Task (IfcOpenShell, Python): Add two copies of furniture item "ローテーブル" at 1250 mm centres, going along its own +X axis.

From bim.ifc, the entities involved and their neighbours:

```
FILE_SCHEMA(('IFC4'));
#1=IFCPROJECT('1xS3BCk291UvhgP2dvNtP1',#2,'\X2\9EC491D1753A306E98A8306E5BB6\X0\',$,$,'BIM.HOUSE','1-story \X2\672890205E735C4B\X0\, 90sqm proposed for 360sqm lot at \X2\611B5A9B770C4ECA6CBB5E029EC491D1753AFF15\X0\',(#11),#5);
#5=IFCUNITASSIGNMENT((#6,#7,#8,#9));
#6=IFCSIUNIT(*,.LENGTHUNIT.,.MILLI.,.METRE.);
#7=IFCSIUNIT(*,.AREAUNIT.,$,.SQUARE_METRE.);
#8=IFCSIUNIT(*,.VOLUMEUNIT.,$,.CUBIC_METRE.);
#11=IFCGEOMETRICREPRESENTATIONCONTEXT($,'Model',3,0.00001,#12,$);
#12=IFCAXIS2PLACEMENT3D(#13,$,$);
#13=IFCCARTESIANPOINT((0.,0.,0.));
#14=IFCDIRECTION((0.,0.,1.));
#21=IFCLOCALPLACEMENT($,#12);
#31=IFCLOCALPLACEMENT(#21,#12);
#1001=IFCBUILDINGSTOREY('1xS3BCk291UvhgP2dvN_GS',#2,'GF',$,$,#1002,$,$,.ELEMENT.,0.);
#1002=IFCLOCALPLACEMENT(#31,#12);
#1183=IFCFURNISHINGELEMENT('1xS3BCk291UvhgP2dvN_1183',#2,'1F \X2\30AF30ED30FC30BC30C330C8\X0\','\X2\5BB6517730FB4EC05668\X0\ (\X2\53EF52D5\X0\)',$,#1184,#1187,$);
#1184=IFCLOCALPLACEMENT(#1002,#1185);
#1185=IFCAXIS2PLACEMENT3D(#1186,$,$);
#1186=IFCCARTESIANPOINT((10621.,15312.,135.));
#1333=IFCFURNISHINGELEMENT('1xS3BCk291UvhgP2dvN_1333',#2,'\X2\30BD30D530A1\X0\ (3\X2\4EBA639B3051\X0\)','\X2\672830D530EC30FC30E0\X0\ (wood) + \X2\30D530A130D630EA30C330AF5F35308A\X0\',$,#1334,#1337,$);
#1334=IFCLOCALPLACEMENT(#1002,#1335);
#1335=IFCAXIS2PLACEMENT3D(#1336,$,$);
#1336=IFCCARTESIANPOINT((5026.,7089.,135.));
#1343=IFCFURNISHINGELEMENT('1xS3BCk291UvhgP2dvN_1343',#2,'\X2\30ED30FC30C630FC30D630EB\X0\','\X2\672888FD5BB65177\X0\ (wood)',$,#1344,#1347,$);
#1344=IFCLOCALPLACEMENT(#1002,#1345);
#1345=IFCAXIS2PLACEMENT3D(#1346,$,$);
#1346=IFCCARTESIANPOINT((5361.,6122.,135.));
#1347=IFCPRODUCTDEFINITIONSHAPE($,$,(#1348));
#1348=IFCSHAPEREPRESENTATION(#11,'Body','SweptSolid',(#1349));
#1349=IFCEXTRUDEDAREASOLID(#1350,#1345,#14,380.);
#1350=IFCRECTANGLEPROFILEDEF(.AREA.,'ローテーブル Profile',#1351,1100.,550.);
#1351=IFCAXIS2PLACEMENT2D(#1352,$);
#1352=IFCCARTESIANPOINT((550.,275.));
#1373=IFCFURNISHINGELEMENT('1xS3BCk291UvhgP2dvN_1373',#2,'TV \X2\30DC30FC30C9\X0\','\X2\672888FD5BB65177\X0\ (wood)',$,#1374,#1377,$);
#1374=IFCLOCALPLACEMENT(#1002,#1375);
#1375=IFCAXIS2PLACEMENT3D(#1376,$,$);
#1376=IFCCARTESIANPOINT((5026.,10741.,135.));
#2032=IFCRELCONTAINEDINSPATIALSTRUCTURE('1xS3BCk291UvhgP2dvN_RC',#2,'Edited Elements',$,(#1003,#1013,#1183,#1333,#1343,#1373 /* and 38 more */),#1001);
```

```python
import ifcopenshell
import ifcopenshell.api.geometry
import ifcopenshell.api.root
import ifcopenshell.util.element
import ifcopenshell.util.placement
import ifcopenshell.util.unit

model = ifcopenshell.open("bim.ifc")
unit_scale = ifcopenshell.util.unit.calculate_unit_scale(model)


def reuse_history(source, copy):
    """copy_class also copies each property set's owner history, people and application; keep the originals."""
    for rel in copy.IsDefinedBy:
        if rel.is_a("IfcRelDefinesByProperties") and (history := rel.RelatingPropertyDefinition.OwnerHistory):
            rel.RelatingPropertyDefinition.OwnerHistory = source.OwnerHistory
            ifcopenshell.util.element.remove_deep2(model, history)


source = model.by_id(1343)
base = ifcopenshell.util.placement.get_local_placement(source.ObjectPlacement)
step = base[:3, 0] * 1.25 / unit_scale

for i in range(1, 3):
    copy = ifcopenshell.api.root.copy_class(model, product=source)
    copy.Representation = ifcopenshell.util.element.copy_deep(
        model, source.Representation, exclude=["IfcGeometricRepresentationContext", "IfcRepresentationMap"]
    )
    reuse_history(source, copy)
    matrix = base.copy()
    matrix[:3, 3] += i * step
    print("added at", matrix[:3, 3].round(3) + 0.0)
    ifcopenshell.api.geometry.edit_object_placement(model, product=copy, matrix=matrix, is_si=False)

model.write("bim_edited.ifc")
```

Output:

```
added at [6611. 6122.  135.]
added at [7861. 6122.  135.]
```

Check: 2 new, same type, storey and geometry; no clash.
